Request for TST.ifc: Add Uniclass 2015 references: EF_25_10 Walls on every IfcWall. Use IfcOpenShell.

First a look at what the model holds.

```python
import ifcopenshell

model = ifcopenshell.open("TST.ifc")
print(model.schema)
print("classifications:", [c.Name for c in model.by_type("IfcClassification")])
for ifc_class in ("IfcDoor", "IfcRoof", "IfcStair", "IfcWall", "IfcWindow"):
    print(ifc_class, len(model.by_type(ifc_class)))
```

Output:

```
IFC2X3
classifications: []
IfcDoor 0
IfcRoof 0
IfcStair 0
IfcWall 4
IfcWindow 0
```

```python
import ifcopenshell
import ifcopenshell.api.classification

model = ifcopenshell.open("TST.ifc")

# IFC2X3 requires Source and Edition and has no link from the project to the system.
system = model.create_entity("IfcClassification", Source="NBS", Edition="2015", Name="Uniclass 2015")

codes = {
    "IfcWall": ("EF_25_10", "Walls"),
}
for ifc_class, (code, name) in codes.items():
    products = model.by_type(ifc_class)
    ifcopenshell.api.classification.add_reference(
        model, products=products, classification=system, identification=code, name=name
    )
    print(code, len(products))

model.write("TST_v2.ifc")
```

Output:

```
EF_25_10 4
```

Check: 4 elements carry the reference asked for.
